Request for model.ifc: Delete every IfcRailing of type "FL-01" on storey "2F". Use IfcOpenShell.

First a look at what the model holds.

```python
import ifcopenshell
import ifcopenshell.util.element

model = ifcopenshell.open("model.ifc")
print(model.schema)
storey = next(s for s in model.by_type("IfcBuildingStorey") if s.Name == "2F")
railings = [e for e in ifcopenshell.util.element.get_decomposition(storey) if e.is_a("IfcRailing")]
seen = {}
for e in railings:
    element_type = ifcopenshell.util.element.get_type(e)
    name = element_type.Name if element_type not in (None, e) else None
    seen[name] = seen.get(name, 0) + 1
for name, count in sorted(seen.items(), key=str):
    print(count, "x", name)
```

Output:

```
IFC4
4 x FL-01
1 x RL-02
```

```python
import ifcopenshell
import ifcopenshell.api.root
import ifcopenshell.util.element

model = ifcopenshell.open("model.ifc")

storey = next(s for s in model.by_type("IfcBuildingStorey") if s.Name == "2F")
railings = [e for e in ifcopenshell.util.element.get_decomposition(storey) if e.is_a("IfcRailing")]
targets = [e for e in railings if (t := ifcopenshell.util.element.get_type(e)) not in (None, e) and t.Name == "FL-01"]

for e in targets:
    ifcopenshell.api.root.remove_product(model, product=e)
print(len(targets), "removed")

model.write("model_edited.ifc")
```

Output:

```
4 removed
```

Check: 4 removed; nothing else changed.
